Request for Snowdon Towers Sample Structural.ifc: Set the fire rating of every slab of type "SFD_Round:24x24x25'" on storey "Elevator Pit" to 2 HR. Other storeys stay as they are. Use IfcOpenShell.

First a look at what the model holds.

```python
import ifcopenshell
import ifcopenshell.util.element

model = ifcopenshell.open("Snowdon Towers Sample Structural.ifc")
print(model.schema)
storey = next(s for s in model.by_type("IfcBuildingStorey") if s.Name == "Elevator Pit")
slabs = [e for e in ifcopenshell.util.element.get_decomposition(storey) if e.is_a("IfcSlab")]
seen = {}
for e in slabs:
    element_type = ifcopenshell.util.element.get_type(e)
    key = (element_type.Name if element_type != e and element_type else None, ifcopenshell.util.element.get_pset(e, "Pset_SlabCommon", "FireRating"))
    seen[key] = seen.get(key, 0) + 1
for (name, value), count in sorted(seen.items(), key=str):
    print(count, "x", name, "|", value)
```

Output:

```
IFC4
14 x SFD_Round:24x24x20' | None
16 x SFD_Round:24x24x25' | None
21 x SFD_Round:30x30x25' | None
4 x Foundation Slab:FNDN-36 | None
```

```python
import ifcopenshell
import ifcopenshell.api.pset
import ifcopenshell.util.element

model = ifcopenshell.open("Snowdon Towers Sample Structural.ifc")

storey = next(s for s in model.by_type("IfcBuildingStorey") if s.Name == "Elevator Pit")
slabs = [e for e in ifcopenshell.util.element.get_decomposition(storey) if e.is_a("IfcSlab")]

count = 0
for e in slabs:
    element_type = ifcopenshell.util.element.get_type(e)
    if element_type in (None, e) or element_type.Name != "SFD_Round:24x24x25'":
        continue
    # add_pset returns the element's existing set when there is one.
    pset = ifcopenshell.api.pset.add_pset(model, product=e, name="Pset_SlabCommon")
    ifcopenshell.api.pset.edit_pset(model, pset=pset, properties={"FireRating": "2 HR"})
    count += 1

print(count, "slabs updated")

model.write("Snowdon Towers Sample Structural_edited.ifc")
```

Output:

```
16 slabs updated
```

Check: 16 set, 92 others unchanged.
